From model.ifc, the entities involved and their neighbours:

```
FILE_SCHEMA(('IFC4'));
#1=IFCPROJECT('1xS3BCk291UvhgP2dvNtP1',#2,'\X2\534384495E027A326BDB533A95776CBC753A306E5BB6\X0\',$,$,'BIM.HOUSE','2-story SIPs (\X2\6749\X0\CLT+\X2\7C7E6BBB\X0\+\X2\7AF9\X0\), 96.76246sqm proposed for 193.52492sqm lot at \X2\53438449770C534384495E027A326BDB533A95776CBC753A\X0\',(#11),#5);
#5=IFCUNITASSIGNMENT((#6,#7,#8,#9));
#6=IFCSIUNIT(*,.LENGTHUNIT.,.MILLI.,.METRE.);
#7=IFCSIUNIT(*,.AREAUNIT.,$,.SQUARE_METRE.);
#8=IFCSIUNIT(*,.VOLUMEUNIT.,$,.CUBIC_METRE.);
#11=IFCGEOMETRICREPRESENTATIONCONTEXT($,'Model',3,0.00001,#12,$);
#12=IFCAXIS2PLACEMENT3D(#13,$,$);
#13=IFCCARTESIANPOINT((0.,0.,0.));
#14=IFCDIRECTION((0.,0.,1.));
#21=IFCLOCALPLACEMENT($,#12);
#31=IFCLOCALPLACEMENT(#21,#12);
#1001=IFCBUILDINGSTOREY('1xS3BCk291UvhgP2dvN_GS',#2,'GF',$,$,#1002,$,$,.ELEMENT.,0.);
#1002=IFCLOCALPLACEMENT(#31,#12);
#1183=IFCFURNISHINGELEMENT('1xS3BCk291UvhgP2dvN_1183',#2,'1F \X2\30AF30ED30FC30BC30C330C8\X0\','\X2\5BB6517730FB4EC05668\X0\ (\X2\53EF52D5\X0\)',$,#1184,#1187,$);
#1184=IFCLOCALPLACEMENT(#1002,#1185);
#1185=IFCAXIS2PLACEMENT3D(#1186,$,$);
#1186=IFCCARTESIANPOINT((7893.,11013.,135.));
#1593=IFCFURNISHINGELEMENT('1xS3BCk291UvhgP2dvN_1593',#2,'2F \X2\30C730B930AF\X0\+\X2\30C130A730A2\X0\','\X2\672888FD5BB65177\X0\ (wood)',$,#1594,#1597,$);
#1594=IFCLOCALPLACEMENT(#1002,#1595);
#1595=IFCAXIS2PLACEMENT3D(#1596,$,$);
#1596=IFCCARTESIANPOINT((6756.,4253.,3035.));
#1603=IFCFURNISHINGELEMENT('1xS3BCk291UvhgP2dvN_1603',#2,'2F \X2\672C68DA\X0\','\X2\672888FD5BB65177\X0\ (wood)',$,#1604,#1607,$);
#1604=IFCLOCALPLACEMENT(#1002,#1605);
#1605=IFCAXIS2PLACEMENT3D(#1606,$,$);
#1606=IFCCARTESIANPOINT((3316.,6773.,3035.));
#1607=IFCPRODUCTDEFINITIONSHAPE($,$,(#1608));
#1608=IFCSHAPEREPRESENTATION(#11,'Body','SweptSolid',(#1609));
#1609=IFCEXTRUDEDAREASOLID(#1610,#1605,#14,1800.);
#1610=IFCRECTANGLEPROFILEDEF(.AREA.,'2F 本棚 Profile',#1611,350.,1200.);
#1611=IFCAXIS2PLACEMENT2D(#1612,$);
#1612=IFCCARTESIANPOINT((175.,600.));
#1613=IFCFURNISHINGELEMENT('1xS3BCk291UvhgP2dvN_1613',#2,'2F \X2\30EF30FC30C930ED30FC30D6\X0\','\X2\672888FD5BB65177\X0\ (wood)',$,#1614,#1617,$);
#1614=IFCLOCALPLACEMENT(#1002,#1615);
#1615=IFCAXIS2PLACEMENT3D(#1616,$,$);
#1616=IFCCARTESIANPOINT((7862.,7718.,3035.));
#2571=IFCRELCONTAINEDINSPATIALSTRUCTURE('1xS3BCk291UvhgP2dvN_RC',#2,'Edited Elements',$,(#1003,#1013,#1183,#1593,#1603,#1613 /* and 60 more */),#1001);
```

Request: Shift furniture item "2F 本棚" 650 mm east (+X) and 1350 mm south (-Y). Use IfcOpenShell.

```python
import ifcopenshell
import ifcopenshell.api.geometry
import ifcopenshell.util.placement
import ifcopenshell.util.unit

model = ifcopenshell.open("model.ifc")
unit_scale = ifcopenshell.util.unit.calculate_unit_scale(model)

item = model.by_guid("1xS3BCk291UvhgP2dvN_1603")
matrix = ifcopenshell.util.placement.get_local_placement(item.ObjectPlacement)
matrix[0, 3] += 0.65 / unit_scale
matrix[1, 3] -= 1.35 / unit_scale
ifcopenshell.api.geometry.edit_object_placement(model, product=item, matrix=matrix, is_si=False)

print(ifcopenshell.util.placement.get_local_placement(item.ObjectPlacement).round(3) + 0.0)

model.write("model-out.ifc")
```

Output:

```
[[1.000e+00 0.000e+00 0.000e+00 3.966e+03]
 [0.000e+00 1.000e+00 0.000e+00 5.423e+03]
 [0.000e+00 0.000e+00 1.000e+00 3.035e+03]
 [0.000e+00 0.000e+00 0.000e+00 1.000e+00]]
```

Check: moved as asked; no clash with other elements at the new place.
